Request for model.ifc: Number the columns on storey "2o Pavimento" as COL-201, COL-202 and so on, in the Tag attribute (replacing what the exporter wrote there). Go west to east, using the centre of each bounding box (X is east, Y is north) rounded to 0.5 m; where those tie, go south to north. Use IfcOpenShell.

First a look at what the model holds.

```python
import ifcopenshell
import ifcopenshell.util.element
import ifcopenshell.util.placement

model = ifcopenshell.open("model.ifc")
print(model.schema)
storey = next(s for s in model.by_type("IfcBuildingStorey") if s.Name == "2o Pavimento")
columns = [e for e in ifcopenshell.util.element.get_decomposition(storey) if e.is_a("IfcColumn")]
for e in sorted(columns, key=lambda e: e.id()):
    origin = ifcopenshell.util.placement.get_local_placement(e.ObjectPlacement)[:3, 3]
    print(e.id(), e.Tag, e.Name, origin.round(2) + 0.0, sep=" | ")
```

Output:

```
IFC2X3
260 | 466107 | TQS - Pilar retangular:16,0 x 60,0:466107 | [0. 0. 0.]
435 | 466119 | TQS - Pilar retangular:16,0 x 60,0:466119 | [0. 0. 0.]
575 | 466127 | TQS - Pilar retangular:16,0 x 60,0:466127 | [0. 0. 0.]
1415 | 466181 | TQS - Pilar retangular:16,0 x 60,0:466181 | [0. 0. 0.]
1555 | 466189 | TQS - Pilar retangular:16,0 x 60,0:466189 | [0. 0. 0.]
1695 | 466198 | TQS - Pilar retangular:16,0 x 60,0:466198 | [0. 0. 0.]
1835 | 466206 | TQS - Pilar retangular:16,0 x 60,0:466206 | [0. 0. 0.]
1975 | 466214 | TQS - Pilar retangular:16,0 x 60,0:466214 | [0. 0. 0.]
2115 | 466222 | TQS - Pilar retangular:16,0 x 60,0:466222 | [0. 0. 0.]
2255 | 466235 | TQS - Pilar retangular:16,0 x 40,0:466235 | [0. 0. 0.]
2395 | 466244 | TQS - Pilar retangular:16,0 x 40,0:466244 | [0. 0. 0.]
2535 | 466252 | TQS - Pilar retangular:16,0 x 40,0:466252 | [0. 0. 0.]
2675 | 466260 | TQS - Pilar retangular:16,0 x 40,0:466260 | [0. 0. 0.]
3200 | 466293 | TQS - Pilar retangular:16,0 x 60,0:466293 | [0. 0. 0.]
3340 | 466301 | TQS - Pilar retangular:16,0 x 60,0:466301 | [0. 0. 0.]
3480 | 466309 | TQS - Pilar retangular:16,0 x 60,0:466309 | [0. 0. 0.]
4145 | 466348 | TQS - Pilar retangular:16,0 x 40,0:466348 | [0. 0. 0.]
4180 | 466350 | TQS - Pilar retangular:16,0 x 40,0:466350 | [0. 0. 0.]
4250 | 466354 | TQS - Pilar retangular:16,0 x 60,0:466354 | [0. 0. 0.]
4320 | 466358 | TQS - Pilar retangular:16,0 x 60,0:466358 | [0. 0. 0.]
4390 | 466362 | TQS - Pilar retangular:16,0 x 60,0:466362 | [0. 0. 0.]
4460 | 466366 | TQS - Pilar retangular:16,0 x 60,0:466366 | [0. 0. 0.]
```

```python
import ifcopenshell
import ifcopenshell.geom
import ifcopenshell.util.element
import ifcopenshell.util.shape

model = ifcopenshell.open("model.ifc")
settings = ifcopenshell.geom.settings()
settings.set("use-world-coords", True)


def centre(element):
    shape = ifcopenshell.geom.create_shape(settings, element)
    return ifcopenshell.util.shape.get_bbox_centroid(shape.geometry)


storey = next(s for s in model.by_type("IfcBuildingStorey") if s.Name == "2o Pavimento")
columns = [e for e in ifcopenshell.util.element.get_decomposition(storey) if e.is_a("IfcColumn")]

# Insertion points can sit at a corner or the storey origin, so sort by the geometry (in metres).
centres = {e: centre(e) for e in columns}
columns.sort(key=lambda e: (round(centres[e][0] / 0.5), centres[e][1]))

for i, e in enumerate(columns, start=1):
    number = f"COL-2{i:02d}"
    e.Tag = number
    print(e.id(), number)

model.write("model_rev.ifc")
```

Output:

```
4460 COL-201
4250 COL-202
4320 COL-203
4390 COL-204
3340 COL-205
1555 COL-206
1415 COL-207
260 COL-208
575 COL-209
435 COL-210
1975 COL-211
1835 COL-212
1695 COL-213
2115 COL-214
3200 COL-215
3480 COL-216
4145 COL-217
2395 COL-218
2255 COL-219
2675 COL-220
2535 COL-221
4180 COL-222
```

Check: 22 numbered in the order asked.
